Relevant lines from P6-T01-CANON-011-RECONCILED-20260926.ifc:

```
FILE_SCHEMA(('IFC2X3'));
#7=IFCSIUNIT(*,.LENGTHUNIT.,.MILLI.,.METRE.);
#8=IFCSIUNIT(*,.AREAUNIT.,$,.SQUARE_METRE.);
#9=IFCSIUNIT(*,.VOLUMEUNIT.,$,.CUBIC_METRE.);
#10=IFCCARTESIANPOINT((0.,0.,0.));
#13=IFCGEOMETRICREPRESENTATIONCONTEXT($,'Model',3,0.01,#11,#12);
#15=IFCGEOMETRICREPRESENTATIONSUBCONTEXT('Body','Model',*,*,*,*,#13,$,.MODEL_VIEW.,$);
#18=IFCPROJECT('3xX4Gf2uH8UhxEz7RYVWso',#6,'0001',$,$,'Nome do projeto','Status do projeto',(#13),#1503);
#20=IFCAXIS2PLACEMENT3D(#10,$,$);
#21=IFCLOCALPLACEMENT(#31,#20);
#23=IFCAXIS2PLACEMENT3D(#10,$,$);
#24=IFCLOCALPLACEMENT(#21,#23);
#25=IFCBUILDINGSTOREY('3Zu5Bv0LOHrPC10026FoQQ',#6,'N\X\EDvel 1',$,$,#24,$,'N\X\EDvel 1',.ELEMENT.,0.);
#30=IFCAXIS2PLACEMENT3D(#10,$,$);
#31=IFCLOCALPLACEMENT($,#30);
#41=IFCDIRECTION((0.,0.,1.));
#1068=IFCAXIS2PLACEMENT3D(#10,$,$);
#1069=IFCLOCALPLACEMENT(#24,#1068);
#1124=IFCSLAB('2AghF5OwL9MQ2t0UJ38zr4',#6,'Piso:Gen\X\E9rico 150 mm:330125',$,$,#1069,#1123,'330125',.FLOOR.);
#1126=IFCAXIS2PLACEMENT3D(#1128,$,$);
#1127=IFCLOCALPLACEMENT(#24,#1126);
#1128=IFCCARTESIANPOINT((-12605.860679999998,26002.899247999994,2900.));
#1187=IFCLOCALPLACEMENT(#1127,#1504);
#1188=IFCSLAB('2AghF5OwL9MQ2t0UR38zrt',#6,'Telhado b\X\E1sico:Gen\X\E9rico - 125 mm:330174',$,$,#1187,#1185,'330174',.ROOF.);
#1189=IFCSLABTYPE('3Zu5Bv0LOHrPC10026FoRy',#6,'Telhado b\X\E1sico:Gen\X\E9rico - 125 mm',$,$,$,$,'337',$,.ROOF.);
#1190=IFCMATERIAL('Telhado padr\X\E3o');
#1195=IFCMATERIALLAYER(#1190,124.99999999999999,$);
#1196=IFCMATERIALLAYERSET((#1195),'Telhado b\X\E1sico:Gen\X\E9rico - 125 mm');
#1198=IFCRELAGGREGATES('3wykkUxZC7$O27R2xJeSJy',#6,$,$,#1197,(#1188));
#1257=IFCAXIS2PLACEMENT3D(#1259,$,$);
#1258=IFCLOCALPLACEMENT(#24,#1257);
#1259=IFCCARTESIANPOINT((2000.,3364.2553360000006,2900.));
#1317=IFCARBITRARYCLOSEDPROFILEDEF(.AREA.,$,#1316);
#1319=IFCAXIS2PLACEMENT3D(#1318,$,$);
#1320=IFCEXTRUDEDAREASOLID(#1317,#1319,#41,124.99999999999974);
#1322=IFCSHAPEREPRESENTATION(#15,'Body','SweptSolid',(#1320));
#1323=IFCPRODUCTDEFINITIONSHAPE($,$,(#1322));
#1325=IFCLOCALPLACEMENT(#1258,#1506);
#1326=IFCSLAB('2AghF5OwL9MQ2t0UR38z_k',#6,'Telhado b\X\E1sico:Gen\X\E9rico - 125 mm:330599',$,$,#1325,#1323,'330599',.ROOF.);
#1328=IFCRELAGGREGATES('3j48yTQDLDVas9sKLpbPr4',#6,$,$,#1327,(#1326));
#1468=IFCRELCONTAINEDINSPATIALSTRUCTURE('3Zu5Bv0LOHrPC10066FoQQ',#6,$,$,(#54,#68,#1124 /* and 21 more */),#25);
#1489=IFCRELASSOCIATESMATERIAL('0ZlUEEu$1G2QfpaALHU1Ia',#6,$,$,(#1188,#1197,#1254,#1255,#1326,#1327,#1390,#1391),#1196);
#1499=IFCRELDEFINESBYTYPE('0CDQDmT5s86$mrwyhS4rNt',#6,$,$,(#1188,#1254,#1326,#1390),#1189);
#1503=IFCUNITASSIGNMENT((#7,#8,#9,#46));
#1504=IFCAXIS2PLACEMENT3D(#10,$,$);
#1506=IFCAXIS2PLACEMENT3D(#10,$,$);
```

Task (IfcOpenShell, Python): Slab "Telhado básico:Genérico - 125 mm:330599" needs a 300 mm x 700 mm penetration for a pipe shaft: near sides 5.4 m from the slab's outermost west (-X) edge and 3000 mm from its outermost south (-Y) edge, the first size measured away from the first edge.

```python
import numpy as np
import ifcopenshell
import ifcopenshell.api.feature
import ifcopenshell.api.geometry
import ifcopenshell.api.root
import ifcopenshell.geom
import ifcopenshell.util.placement
import ifcopenshell.util.representation
import ifcopenshell.util.shape
import ifcopenshell.util.unit

model = ifcopenshell.open("P6-T01-CANON-011-RECONCILED-20260926.ifc")
unit_scale = ifcopenshell.util.unit.calculate_unit_scale(model)
settings = ifcopenshell.geom.settings()


def volume(element):
    """Net volume in cubic metres, openings subtracted."""
    shape = ifcopenshell.geom.create_shape(settings, element)
    return ifcopenshell.util.shape.get_volume(shape.geometry)


slab = model.by_id(1326)
before = volume(slab)

# Extent in the slab's own axes, in metres. The edges named are its -X and -Y sides.
slab_shape = ifcopenshell.geom.create_shape(settings, slab)
vertices = ifcopenshell.util.shape.get_vertices(slab_shape.geometry)
x_min, y_min, bottom = vertices.min(axis=0)
top = vertices[:, 2].max()

opening = ifcopenshell.api.root.create_entity(model, ifc_class="IfcOpeningElement", name="Pipe shaft opening")
context = ifcopenshell.util.representation.get_context(model, "Model", "Body", "MODEL_VIEW")
width, depth = 0.3, 0.7
outline = [(0.0, 0.0), (width, 0.0), (width, depth), (0.0, depth), (0.0, 0.0)]
# Overshoot both faces by 50 mm so the cut is clean.
shape = ifcopenshell.api.geometry.add_slab_representation(
    model, context=context, depth=top - bottom + 0.1, polyline=outline
)
ifcopenshell.api.geometry.assign_representation(model, product=opening, representation=shape)

matrix = ifcopenshell.util.placement.get_local_placement(slab.ObjectPlacement)
matrix[:, 3] = matrix @ np.append(np.array([x_min + 5.4, y_min + 3, bottom - 0.05]) / unit_scale, 1.0)
ifcopenshell.api.geometry.edit_object_placement(model, product=opening, matrix=matrix, is_si=False)
ifcopenshell.api.feature.add_feature(model, feature=opening, element=slab)

after = volume(slab)

print(f"slab volume {before:.3f} -> {after:.3f} m3")

model.write("P6-T01-CANON-011-RECONCILED-20260926_rev.ifc")
```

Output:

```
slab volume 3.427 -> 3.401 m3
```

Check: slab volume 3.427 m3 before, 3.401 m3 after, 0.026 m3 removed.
